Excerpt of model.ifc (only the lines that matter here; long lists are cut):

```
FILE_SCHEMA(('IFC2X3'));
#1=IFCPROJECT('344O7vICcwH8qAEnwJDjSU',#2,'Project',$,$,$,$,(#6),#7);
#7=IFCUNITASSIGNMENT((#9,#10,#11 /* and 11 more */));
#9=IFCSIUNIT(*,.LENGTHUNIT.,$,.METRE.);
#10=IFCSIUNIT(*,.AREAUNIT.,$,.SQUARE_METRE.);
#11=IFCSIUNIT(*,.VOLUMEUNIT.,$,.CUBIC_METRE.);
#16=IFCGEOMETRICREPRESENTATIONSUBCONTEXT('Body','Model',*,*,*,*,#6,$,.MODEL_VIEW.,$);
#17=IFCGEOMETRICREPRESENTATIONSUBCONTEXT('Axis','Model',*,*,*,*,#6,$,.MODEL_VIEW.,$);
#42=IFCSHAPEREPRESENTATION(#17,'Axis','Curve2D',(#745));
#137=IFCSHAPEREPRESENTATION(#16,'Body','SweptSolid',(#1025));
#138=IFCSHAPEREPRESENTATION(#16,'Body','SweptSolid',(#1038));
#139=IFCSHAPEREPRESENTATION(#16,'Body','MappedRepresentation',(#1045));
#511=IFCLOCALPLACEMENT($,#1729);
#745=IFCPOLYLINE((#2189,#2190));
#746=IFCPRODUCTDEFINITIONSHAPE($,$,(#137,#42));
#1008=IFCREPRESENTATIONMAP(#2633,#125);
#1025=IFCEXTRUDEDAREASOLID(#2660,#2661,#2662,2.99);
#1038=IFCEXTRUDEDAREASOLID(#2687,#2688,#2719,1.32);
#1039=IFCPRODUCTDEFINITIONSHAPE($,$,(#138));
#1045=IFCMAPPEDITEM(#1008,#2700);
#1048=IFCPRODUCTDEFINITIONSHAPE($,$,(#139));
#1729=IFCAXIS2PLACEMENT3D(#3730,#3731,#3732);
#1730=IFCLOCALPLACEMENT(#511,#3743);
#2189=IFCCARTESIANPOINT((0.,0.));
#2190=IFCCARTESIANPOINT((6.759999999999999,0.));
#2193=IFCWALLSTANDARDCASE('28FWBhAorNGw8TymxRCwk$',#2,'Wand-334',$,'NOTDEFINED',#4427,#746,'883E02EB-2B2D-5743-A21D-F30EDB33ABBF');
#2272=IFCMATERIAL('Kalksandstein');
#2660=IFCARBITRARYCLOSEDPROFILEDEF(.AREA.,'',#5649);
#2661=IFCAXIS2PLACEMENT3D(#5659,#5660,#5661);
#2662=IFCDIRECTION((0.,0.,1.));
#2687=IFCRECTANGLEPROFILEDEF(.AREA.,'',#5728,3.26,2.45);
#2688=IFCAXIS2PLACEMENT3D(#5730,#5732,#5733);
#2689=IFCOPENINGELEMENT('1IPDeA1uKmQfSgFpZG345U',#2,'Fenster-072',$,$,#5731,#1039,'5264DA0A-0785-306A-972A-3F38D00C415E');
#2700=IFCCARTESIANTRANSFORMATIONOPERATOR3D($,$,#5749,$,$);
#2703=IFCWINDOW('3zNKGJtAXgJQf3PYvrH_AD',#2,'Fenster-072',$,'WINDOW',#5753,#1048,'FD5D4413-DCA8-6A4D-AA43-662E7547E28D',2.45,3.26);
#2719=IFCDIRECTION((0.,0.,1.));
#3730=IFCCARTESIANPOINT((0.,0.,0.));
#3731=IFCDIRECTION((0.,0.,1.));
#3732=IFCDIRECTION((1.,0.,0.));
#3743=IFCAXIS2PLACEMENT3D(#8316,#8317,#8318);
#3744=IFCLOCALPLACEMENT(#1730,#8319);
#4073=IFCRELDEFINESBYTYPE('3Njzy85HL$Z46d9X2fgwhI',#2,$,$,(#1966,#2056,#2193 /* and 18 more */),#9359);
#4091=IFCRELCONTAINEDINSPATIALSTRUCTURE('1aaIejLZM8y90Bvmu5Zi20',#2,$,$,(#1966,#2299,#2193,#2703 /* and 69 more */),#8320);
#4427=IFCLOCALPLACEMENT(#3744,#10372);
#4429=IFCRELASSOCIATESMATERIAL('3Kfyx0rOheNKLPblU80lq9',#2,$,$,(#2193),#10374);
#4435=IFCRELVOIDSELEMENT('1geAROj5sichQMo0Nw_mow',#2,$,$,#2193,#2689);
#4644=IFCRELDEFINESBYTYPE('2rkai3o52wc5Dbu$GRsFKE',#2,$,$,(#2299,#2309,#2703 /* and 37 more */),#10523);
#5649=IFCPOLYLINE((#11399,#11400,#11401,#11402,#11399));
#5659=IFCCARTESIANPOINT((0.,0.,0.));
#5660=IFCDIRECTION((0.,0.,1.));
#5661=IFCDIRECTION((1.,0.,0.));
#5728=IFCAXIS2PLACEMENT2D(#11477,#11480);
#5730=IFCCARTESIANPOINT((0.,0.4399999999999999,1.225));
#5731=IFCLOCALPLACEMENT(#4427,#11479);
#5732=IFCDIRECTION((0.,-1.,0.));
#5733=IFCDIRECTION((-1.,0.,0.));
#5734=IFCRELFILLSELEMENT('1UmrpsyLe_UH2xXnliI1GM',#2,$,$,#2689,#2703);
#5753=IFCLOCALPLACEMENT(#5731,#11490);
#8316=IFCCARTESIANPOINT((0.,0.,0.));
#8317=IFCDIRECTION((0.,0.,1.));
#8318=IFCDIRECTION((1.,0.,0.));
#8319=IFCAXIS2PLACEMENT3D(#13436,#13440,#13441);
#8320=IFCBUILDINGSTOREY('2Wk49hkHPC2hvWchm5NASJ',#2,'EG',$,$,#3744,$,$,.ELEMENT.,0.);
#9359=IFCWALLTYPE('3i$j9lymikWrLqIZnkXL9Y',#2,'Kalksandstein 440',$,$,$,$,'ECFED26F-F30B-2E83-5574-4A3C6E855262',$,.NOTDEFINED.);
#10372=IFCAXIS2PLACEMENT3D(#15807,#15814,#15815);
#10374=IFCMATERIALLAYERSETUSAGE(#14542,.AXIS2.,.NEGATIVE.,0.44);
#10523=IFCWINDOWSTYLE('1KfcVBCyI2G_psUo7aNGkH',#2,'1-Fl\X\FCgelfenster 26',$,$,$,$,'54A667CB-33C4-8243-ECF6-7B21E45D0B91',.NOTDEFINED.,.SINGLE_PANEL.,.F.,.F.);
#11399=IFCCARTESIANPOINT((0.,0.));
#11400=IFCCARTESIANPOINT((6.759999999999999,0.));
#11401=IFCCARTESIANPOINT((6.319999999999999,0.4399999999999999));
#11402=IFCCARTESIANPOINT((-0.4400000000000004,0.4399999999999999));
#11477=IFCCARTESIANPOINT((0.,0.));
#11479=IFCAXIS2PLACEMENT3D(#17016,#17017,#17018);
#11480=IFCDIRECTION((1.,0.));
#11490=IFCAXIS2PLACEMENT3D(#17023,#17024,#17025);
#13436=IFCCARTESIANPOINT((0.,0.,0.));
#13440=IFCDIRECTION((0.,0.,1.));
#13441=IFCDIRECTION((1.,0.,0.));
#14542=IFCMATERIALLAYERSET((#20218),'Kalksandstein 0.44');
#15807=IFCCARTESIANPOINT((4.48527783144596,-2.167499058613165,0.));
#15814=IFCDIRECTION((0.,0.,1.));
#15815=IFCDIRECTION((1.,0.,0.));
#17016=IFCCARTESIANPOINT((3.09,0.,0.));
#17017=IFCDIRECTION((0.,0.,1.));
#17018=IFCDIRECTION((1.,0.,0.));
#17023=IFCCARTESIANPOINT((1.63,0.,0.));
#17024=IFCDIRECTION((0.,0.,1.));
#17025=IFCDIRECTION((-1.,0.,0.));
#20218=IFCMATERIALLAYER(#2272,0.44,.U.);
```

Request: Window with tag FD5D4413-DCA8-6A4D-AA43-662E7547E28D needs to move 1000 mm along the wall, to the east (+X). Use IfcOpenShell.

```python
import ifcopenshell
import ifcopenshell.api.geometry
import ifcopenshell.util.placement

model = ifcopenshell.open("model.ifc")

window = model.by_id(2703)
opening = window.FillsVoids[0].RelatingOpeningElement
wall = opening.VoidsElements[0].RelatingBuildingElement

wall_matrix = ifcopenshell.util.placement.get_local_placement(wall.ObjectPlacement)
shift = wall_matrix[:3, 0] * 1.0
before = ifcopenshell.util.placement.get_local_placement(window.ObjectPlacement)[:3, 3].copy()

# The window is placed relative to its opening, so it follows when the opening moves.
matrix = ifcopenshell.util.placement.get_local_placement(opening.ObjectPlacement)
matrix[:3, 3] += shift
ifcopenshell.api.geometry.edit_object_placement(
    model, product=opening, matrix=matrix, is_si=False, should_transform_children=True
)

after = ifcopenshell.util.placement.get_local_placement(window.ObjectPlacement)[:3, 3]
print("window moved by", (after - before).round(3) + 0.0)

model.write("model_rev.ifc")
```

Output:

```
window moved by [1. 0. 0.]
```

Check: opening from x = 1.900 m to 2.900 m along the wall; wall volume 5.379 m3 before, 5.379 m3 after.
